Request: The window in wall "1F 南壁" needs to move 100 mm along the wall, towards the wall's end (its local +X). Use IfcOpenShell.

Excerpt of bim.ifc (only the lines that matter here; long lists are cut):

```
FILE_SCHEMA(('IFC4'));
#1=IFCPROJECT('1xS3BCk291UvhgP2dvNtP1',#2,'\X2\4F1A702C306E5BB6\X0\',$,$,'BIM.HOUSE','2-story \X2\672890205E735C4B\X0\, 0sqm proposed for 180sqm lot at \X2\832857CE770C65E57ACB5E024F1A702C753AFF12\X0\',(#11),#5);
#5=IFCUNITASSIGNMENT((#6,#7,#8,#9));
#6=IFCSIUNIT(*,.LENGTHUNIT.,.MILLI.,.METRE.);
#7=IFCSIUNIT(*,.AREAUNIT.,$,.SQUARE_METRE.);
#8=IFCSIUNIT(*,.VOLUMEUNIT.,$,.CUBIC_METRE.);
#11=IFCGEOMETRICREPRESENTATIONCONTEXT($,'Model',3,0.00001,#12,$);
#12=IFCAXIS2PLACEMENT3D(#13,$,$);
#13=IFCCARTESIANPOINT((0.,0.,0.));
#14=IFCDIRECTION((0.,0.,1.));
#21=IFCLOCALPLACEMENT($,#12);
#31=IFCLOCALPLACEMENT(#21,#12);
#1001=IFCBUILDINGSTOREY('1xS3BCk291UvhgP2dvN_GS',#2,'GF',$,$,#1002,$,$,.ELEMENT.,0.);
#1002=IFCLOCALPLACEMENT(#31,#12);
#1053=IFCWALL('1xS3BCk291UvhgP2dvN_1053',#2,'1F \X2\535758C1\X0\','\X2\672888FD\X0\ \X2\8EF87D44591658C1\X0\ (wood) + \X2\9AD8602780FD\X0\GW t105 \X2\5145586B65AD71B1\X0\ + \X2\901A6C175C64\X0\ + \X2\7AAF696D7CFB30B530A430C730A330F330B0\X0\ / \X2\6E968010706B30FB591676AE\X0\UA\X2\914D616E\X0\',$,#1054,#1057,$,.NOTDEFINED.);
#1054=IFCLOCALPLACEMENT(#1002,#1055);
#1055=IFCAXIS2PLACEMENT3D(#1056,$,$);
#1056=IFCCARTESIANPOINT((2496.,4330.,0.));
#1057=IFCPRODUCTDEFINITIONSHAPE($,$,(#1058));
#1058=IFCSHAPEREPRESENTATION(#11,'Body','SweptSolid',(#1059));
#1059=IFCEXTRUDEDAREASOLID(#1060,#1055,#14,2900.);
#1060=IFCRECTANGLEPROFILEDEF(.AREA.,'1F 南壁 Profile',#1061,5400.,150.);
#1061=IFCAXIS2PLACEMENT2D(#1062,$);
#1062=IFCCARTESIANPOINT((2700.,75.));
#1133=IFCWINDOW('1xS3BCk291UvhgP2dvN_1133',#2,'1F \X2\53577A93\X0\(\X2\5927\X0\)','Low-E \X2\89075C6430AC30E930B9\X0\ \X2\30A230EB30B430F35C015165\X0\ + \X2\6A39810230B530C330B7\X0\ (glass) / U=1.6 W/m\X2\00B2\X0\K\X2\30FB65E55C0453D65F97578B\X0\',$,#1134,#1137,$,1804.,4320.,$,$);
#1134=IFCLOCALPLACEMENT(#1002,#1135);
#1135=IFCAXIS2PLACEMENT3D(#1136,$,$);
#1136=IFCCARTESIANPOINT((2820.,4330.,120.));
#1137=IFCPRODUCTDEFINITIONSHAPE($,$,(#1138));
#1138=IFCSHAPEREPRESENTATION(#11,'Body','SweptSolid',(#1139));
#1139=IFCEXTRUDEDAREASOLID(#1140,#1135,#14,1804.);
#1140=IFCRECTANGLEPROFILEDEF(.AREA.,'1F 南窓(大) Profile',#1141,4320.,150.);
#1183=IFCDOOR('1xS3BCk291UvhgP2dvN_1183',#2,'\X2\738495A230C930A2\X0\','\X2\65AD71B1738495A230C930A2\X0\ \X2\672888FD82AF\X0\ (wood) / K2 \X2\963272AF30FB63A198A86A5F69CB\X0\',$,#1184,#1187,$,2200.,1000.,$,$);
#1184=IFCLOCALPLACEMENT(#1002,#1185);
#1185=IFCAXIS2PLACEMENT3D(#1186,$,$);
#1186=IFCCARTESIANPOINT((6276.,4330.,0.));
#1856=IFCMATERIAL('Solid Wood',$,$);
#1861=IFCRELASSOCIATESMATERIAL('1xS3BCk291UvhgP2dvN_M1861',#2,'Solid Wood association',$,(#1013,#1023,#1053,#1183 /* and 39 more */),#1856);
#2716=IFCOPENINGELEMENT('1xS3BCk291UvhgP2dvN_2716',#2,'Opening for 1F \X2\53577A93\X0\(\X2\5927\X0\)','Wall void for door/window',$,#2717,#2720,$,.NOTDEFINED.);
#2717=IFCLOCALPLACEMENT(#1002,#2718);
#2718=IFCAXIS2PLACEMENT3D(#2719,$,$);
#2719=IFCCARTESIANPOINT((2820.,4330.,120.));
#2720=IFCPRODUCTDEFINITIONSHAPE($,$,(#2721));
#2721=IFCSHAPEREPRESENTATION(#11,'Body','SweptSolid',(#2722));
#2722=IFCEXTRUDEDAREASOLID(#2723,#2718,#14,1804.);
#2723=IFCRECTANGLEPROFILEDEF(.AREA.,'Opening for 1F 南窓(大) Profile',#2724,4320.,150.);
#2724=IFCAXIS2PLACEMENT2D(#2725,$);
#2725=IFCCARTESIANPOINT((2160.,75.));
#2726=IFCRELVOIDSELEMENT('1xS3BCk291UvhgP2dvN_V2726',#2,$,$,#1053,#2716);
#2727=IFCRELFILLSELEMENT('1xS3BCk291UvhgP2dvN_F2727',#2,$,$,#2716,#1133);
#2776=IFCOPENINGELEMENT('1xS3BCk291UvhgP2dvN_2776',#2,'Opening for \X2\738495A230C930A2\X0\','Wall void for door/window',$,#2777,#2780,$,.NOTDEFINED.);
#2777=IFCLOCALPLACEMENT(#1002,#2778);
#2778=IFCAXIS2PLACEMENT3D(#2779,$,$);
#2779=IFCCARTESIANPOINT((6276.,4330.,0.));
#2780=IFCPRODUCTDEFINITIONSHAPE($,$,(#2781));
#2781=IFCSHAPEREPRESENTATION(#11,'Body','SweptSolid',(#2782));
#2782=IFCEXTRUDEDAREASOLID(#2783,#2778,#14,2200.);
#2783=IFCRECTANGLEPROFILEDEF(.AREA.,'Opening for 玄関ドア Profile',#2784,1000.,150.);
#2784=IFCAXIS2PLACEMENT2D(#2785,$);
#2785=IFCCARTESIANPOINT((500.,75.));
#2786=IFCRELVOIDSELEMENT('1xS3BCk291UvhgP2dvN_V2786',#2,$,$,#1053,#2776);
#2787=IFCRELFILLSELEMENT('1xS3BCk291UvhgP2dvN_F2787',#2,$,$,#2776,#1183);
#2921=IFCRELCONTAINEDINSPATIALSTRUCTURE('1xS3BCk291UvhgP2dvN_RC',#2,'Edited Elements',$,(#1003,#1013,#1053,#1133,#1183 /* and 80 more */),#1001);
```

```python
import ifcopenshell
import ifcopenshell.api.geometry
import ifcopenshell.util.placement

model = ifcopenshell.open("bim.ifc")

window = model.by_guid("1xS3BCk291UvhgP2dvN_1133")
opening = window.FillsVoids[0].RelatingOpeningElement
wall = opening.VoidsElements[0].RelatingBuildingElement

wall_matrix = ifcopenshell.util.placement.get_local_placement(wall.ObjectPlacement)
shift = wall_matrix[:3, 0] * 100.0
before = ifcopenshell.util.placement.get_local_placement(window.ObjectPlacement)[:3, 3].copy()

# The window is not placed relative to its opening, so move both.
for product in (opening, window):
    matrix = ifcopenshell.util.placement.get_local_placement(product.ObjectPlacement)
    matrix[:3, 3] += shift
    ifcopenshell.api.geometry.edit_object_placement(model, product=product, matrix=matrix, is_si=False)

after = ifcopenshell.util.placement.get_local_placement(window.ObjectPlacement)[:3, 3]
print("window moved by", (after - before).round(3) + 0.0)

model.write("bim_updated.ifc")
```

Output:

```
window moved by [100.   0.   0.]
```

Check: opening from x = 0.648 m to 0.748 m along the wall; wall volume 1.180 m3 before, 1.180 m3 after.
